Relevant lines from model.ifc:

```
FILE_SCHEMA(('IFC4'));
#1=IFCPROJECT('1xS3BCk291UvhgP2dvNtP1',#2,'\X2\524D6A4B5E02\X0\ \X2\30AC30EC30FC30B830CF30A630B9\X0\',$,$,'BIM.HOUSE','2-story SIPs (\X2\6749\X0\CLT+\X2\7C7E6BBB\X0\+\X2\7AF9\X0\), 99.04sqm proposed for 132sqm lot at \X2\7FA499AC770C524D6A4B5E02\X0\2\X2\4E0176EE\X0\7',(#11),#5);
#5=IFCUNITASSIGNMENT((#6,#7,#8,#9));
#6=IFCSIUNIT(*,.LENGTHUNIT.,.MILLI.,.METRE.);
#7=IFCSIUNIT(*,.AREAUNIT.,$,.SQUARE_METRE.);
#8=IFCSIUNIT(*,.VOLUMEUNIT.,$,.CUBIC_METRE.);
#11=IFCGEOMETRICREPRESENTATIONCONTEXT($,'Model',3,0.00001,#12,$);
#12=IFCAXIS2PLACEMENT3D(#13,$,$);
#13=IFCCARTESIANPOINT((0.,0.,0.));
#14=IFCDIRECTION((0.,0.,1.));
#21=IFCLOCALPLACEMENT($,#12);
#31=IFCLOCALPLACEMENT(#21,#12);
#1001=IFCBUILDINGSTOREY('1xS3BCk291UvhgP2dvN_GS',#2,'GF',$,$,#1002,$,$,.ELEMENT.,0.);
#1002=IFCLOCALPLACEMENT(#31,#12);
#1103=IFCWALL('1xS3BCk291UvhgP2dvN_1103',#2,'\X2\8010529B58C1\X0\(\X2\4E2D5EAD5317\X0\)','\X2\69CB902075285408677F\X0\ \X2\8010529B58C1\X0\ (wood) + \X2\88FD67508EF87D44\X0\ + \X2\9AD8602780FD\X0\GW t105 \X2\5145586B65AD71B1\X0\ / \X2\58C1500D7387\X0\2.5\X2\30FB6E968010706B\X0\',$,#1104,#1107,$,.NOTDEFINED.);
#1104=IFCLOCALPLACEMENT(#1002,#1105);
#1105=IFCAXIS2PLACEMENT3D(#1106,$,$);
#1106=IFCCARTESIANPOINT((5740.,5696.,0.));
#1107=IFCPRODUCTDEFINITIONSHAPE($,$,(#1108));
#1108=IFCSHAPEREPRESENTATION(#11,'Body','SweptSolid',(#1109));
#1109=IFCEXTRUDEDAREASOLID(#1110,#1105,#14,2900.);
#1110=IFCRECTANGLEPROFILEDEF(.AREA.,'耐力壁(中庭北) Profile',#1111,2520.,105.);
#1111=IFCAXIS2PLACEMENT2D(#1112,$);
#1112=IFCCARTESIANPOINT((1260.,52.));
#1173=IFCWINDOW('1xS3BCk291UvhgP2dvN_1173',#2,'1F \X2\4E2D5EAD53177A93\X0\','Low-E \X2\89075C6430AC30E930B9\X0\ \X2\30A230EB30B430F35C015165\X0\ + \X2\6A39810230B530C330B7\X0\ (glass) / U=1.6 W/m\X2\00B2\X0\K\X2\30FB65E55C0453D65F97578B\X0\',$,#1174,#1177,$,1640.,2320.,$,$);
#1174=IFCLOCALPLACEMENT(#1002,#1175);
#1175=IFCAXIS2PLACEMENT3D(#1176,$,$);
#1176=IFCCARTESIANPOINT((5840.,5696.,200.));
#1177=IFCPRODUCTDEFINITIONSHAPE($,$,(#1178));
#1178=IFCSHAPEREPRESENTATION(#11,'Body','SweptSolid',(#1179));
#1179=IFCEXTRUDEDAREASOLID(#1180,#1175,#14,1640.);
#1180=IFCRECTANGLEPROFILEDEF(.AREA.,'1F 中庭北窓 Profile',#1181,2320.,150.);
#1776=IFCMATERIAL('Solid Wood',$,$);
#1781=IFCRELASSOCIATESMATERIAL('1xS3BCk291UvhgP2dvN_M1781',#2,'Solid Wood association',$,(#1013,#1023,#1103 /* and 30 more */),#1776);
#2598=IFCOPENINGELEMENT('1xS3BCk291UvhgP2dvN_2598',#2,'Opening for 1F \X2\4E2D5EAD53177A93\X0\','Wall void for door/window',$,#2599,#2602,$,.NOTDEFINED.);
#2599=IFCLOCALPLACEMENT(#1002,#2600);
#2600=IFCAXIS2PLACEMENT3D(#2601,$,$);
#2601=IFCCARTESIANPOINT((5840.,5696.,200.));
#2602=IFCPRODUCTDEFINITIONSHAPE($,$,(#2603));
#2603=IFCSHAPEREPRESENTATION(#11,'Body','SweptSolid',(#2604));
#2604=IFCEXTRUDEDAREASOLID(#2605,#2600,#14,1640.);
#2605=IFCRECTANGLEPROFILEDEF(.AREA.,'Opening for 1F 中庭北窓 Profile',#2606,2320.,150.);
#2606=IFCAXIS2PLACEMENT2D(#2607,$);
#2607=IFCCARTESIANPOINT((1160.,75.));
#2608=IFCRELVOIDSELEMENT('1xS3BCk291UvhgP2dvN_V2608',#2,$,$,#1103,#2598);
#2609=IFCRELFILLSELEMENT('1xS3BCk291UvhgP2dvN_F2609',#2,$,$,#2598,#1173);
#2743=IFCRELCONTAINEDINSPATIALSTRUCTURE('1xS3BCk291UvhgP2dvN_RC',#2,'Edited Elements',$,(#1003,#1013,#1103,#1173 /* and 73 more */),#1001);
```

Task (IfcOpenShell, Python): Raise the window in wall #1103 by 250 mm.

```python
import numpy as np
import ifcopenshell
import ifcopenshell.api.geometry
import ifcopenshell.util.placement
import ifcopenshell.util.unit

model = ifcopenshell.open("model.ifc")
unit_scale = ifcopenshell.util.unit.calculate_unit_scale(model)

window = model.by_guid("1xS3BCk291UvhgP2dvN_1173")
opening = window.FillsVoids[0].RelatingOpeningElement
dz = 0.25 / unit_scale

shift = np.array([0.0, 0.0, dz])
# The window is not placed relative to its opening, so move both.
for product in (opening, window):
    matrix = ifcopenshell.util.placement.get_local_placement(product.ObjectPlacement)
    matrix[:3, 3] += shift
    ifcopenshell.api.geometry.edit_object_placement(model, product=product, matrix=matrix, is_si=False)

print(f"moved by {dz * unit_scale:+.3f} m")

model.write("model_rev.ifc")
```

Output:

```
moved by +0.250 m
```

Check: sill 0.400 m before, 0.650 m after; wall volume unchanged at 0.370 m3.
